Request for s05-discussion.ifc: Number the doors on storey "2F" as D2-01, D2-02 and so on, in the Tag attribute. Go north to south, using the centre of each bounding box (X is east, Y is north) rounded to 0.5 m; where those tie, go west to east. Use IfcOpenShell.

First a look at what the model holds.

```python
import ifcopenshell
import ifcopenshell.util.element
import ifcopenshell.util.placement

model = ifcopenshell.open("s05-discussion.ifc")
print(model.schema)
storey = next(s for s in model.by_type("IfcBuildingStorey") if s.Name == "2F")
doors = [e for e in ifcopenshell.util.element.get_decomposition(storey) if e.is_a("IfcDoor")]
for e in sorted(doors, key=lambda e: e.id()):
    origin = ifcopenshell.util.placement.get_local_placement(e.ObjectPlacement)[:3, 3]
    print(e.id(), e.Tag, e.Name, origin.round(2) + 0.0, sep=" | ")
```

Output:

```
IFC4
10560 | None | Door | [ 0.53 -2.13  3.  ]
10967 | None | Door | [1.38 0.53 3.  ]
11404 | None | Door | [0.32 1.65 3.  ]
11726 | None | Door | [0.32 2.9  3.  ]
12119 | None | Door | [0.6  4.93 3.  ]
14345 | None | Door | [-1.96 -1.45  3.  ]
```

```python
import ifcopenshell
import ifcopenshell.geom
import ifcopenshell.util.element
import ifcopenshell.util.shape

model = ifcopenshell.open("s05-discussion.ifc")
settings = ifcopenshell.geom.settings()
settings.set("use-world-coords", True)


def centre(element):
    shape = ifcopenshell.geom.create_shape(settings, element)
    return ifcopenshell.util.shape.get_bbox_centroid(shape.geometry)


storey = next(s for s in model.by_type("IfcBuildingStorey") if s.Name == "2F")
doors = [e for e in ifcopenshell.util.element.get_decomposition(storey) if e.is_a("IfcDoor")]

# Insertion points can sit at a corner or the storey origin, so sort by the geometry (in metres).
centres = {e: centre(e) for e in doors}
doors.sort(key=lambda e: (-round(centres[e][1] / 0.5), centres[e][0]))

for i, e in enumerate(doors, start=1):
    number = f"D2-{i:02d}"
    e.Tag = number
    print(e.id(), number)

model.write("s05-discussion_v2.ifc")
```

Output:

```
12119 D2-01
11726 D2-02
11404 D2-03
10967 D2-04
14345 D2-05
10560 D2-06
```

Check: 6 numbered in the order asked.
